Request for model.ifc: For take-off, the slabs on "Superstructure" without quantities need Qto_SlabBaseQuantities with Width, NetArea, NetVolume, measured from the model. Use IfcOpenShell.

First a look at what the model holds.

```python
import ifcopenshell
import ifcopenshell.util.element
import ifcopenshell.util.unit

model = ifcopenshell.open("model.ifc")
print(model.schema)
for unit_type in ("LENGTHUNIT", "AREAUNIT", "VOLUMEUNIT"):
    print(unit_type, ifcopenshell.util.unit.calculate_unit_scale(model, unit_type))
storey = next(s for s in model.by_type("IfcBuildingStorey") if s.Name == "Superstructure")
slabs = [e for e in ifcopenshell.util.element.get_decomposition(storey) if e.is_a("IfcSlab")]
for e in sorted(slabs, key=lambda e: e.id()):
    print(e.id(), e.is_a(), e.Name, list(ifcopenshell.util.element.get_psets(e, qtos_only=True)), sep=" | ")
```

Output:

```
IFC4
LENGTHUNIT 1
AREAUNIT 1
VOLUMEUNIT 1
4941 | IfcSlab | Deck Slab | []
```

```python
import ifcopenshell
import ifcopenshell.api.pset
import ifcopenshell.geom
import ifcopenshell.util.element
import ifcopenshell.util.shape
import ifcopenshell.util.unit

model = ifcopenshell.open("model.ifc")
unit_scale = ifcopenshell.util.unit.calculate_unit_scale(model)
area_scale = ifcopenshell.util.unit.calculate_unit_scale(model, "AREAUNIT")
volume_scale = ifcopenshell.util.unit.calculate_unit_scale(model, "VOLUMEUNIT")
settings = ifcopenshell.geom.settings()

storey = next(s for s in model.by_type("IfcBuildingStorey") if s.Name == "Superstructure")
slabs = [e for e in ifcopenshell.util.element.get_decomposition(storey) if e.is_a("IfcSlab")]

for e in sorted(slabs, key=lambda e: e.id()):
    if ifcopenshell.util.element.get_psets(e, qtos_only=True, should_inherit=False):
        continue
    # Geometry comes back in metres, in the element's own axes.
    shape = ifcopenshell.geom.create_shape(settings, e)
    values = {
        "Width": ifcopenshell.util.shape.get_z(shape.geometry) / unit_scale,
        "NetArea": ifcopenshell.util.shape.get_footprint_area(shape.geometry) / area_scale,
        "NetVolume": ifcopenshell.util.shape.get_volume(shape.geometry) / volume_scale,
    }
    qto = ifcopenshell.api.pset.add_qto(model, product=e, name="Qto_SlabBaseQuantities")
    ifcopenshell.api.pset.edit_qto(model, qto=qto, properties=values)
    print(e.id(), {k: round(v, 3) for k, v in values.items()})

model.write("model_edited.ifc")
```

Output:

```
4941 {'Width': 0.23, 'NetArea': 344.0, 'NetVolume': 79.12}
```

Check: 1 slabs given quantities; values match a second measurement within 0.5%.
